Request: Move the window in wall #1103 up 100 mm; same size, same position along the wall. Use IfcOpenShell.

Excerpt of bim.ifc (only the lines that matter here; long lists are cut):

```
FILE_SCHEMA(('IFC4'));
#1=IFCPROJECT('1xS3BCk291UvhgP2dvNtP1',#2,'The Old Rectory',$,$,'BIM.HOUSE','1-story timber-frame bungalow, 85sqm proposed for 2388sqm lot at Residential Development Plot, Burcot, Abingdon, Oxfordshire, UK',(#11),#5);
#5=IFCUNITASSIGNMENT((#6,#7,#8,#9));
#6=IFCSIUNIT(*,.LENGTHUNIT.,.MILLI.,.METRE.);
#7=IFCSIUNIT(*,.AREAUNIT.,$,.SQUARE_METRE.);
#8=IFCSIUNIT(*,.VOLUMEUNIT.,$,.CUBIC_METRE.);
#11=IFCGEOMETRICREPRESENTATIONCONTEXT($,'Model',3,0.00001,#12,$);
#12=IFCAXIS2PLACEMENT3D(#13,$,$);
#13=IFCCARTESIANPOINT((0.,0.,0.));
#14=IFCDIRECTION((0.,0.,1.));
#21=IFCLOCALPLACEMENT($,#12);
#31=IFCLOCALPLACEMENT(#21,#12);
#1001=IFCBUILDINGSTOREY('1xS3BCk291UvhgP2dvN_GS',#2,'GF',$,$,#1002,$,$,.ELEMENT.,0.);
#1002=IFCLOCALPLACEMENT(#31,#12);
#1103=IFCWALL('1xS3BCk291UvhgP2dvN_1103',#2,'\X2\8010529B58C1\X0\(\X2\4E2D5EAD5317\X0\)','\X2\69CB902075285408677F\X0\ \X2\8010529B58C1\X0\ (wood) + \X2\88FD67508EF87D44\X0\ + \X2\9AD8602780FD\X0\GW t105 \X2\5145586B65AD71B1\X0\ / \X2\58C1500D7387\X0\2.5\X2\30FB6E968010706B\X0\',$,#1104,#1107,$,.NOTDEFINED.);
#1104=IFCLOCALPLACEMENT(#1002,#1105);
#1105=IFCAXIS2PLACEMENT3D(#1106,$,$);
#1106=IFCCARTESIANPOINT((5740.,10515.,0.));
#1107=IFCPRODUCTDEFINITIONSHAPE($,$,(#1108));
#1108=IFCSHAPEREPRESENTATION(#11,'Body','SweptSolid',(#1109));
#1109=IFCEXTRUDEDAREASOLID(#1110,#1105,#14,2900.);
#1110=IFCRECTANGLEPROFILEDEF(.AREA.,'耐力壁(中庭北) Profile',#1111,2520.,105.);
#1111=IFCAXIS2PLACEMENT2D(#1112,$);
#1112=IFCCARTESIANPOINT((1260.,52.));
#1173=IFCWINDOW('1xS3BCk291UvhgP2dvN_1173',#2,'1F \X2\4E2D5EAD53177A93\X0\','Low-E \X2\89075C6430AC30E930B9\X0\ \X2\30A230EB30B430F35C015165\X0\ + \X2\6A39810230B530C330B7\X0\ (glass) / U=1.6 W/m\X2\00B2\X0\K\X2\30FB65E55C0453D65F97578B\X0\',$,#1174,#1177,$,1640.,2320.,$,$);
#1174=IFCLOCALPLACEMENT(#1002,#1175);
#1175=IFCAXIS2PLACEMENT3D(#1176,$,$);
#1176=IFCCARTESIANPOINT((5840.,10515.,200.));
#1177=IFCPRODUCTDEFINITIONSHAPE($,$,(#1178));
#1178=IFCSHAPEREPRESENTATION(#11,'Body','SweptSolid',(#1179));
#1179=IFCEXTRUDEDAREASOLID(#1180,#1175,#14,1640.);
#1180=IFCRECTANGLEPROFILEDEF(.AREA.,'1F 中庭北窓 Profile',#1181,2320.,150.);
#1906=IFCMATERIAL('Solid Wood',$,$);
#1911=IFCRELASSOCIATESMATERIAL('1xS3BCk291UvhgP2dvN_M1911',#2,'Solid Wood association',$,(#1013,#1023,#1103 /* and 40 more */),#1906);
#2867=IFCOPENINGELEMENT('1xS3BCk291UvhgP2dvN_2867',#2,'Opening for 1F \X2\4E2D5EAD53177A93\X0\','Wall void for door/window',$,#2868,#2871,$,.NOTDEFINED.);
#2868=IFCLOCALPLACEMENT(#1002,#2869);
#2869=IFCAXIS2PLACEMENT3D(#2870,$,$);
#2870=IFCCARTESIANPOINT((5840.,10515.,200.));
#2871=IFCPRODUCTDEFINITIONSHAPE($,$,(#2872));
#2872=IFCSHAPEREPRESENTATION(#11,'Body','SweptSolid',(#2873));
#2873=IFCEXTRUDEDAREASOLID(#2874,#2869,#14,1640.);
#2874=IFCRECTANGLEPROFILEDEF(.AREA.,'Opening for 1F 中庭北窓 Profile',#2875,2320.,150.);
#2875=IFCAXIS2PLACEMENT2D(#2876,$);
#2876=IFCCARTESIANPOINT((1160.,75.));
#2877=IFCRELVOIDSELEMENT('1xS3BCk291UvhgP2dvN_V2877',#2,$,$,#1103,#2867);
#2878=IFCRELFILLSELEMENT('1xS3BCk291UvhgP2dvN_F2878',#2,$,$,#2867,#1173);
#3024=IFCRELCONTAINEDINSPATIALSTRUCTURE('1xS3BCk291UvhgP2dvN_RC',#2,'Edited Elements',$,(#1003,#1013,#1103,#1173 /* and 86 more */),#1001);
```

```python
import numpy as np
import ifcopenshell
import ifcopenshell.api.geometry
import ifcopenshell.util.placement
import ifcopenshell.util.unit

model = ifcopenshell.open("bim.ifc")
unit_scale = ifcopenshell.util.unit.calculate_unit_scale(model)

window = model.by_id(1173)
opening = window.FillsVoids[0].RelatingOpeningElement
dz = 100.0

shift = np.array([0.0, 0.0, dz])
# The window is not placed relative to its opening, so move both.
for product in (opening, window):
    matrix = ifcopenshell.util.placement.get_local_placement(product.ObjectPlacement)
    matrix[:3, 3] += shift
    ifcopenshell.api.geometry.edit_object_placement(model, product=product, matrix=matrix, is_si=False)

print(f"moved by {dz * unit_scale:+.3f} m")

model.write("bim-out.ifc")
```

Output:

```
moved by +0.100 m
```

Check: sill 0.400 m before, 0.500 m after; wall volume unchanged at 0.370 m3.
